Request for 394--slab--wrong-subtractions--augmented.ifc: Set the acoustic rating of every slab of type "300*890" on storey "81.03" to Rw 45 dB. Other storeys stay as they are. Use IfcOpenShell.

First a look at what the model holds.

```python
import ifcopenshell
import ifcopenshell.util.element

model = ifcopenshell.open("394--slab--wrong-subtractions--augmented.ifc")
print(model.schema)
storey = next(s for s in model.by_type("IfcBuildingStorey") if s.Name == "81.03")
slabs = [e for e in ifcopenshell.util.element.get_decomposition(storey) if e.is_a("IfcSlab")]
seen = {}
for e in slabs:
    element_type = ifcopenshell.util.element.get_type(e)
    key = (element_type.Name if element_type != e and element_type else None, ifcopenshell.util.element.get_pset(e, "Pset_SlabCommon", "AcousticRating"))
    seen[key] = seen.get(key, 0) + 1
for (name, value), count in sorted(seen.items(), key=str):
    print(count, "x", name, "|", value)
```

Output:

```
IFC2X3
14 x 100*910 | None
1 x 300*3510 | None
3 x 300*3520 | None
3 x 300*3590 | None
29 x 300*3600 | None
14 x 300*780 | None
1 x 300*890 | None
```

```python
import ifcopenshell
import ifcopenshell.api.pset
import ifcopenshell.util.element

model = ifcopenshell.open("394--slab--wrong-subtractions--augmented.ifc")

storey = next(s for s in model.by_type("IfcBuildingStorey") if s.Name == "81.03")
slabs = [e for e in ifcopenshell.util.element.get_decomposition(storey) if e.is_a("IfcSlab")]

count = 0
for e in slabs:
    element_type = ifcopenshell.util.element.get_type(e)
    if element_type in (None, e) or element_type.Name != "300*890":
        continue
    # add_pset returns the element's existing set when there is one.
    pset = ifcopenshell.api.pset.add_pset(model, product=e, name="Pset_SlabCommon")
    ifcopenshell.api.pset.edit_pset(model, pset=pset, properties={"AcousticRating": "Rw 45 dB"})
    count += 1

print(count, "slabs updated")

model.write("394--slab--wrong-subtractions--augmented-out.ifc")
```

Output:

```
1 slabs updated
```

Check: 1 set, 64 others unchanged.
